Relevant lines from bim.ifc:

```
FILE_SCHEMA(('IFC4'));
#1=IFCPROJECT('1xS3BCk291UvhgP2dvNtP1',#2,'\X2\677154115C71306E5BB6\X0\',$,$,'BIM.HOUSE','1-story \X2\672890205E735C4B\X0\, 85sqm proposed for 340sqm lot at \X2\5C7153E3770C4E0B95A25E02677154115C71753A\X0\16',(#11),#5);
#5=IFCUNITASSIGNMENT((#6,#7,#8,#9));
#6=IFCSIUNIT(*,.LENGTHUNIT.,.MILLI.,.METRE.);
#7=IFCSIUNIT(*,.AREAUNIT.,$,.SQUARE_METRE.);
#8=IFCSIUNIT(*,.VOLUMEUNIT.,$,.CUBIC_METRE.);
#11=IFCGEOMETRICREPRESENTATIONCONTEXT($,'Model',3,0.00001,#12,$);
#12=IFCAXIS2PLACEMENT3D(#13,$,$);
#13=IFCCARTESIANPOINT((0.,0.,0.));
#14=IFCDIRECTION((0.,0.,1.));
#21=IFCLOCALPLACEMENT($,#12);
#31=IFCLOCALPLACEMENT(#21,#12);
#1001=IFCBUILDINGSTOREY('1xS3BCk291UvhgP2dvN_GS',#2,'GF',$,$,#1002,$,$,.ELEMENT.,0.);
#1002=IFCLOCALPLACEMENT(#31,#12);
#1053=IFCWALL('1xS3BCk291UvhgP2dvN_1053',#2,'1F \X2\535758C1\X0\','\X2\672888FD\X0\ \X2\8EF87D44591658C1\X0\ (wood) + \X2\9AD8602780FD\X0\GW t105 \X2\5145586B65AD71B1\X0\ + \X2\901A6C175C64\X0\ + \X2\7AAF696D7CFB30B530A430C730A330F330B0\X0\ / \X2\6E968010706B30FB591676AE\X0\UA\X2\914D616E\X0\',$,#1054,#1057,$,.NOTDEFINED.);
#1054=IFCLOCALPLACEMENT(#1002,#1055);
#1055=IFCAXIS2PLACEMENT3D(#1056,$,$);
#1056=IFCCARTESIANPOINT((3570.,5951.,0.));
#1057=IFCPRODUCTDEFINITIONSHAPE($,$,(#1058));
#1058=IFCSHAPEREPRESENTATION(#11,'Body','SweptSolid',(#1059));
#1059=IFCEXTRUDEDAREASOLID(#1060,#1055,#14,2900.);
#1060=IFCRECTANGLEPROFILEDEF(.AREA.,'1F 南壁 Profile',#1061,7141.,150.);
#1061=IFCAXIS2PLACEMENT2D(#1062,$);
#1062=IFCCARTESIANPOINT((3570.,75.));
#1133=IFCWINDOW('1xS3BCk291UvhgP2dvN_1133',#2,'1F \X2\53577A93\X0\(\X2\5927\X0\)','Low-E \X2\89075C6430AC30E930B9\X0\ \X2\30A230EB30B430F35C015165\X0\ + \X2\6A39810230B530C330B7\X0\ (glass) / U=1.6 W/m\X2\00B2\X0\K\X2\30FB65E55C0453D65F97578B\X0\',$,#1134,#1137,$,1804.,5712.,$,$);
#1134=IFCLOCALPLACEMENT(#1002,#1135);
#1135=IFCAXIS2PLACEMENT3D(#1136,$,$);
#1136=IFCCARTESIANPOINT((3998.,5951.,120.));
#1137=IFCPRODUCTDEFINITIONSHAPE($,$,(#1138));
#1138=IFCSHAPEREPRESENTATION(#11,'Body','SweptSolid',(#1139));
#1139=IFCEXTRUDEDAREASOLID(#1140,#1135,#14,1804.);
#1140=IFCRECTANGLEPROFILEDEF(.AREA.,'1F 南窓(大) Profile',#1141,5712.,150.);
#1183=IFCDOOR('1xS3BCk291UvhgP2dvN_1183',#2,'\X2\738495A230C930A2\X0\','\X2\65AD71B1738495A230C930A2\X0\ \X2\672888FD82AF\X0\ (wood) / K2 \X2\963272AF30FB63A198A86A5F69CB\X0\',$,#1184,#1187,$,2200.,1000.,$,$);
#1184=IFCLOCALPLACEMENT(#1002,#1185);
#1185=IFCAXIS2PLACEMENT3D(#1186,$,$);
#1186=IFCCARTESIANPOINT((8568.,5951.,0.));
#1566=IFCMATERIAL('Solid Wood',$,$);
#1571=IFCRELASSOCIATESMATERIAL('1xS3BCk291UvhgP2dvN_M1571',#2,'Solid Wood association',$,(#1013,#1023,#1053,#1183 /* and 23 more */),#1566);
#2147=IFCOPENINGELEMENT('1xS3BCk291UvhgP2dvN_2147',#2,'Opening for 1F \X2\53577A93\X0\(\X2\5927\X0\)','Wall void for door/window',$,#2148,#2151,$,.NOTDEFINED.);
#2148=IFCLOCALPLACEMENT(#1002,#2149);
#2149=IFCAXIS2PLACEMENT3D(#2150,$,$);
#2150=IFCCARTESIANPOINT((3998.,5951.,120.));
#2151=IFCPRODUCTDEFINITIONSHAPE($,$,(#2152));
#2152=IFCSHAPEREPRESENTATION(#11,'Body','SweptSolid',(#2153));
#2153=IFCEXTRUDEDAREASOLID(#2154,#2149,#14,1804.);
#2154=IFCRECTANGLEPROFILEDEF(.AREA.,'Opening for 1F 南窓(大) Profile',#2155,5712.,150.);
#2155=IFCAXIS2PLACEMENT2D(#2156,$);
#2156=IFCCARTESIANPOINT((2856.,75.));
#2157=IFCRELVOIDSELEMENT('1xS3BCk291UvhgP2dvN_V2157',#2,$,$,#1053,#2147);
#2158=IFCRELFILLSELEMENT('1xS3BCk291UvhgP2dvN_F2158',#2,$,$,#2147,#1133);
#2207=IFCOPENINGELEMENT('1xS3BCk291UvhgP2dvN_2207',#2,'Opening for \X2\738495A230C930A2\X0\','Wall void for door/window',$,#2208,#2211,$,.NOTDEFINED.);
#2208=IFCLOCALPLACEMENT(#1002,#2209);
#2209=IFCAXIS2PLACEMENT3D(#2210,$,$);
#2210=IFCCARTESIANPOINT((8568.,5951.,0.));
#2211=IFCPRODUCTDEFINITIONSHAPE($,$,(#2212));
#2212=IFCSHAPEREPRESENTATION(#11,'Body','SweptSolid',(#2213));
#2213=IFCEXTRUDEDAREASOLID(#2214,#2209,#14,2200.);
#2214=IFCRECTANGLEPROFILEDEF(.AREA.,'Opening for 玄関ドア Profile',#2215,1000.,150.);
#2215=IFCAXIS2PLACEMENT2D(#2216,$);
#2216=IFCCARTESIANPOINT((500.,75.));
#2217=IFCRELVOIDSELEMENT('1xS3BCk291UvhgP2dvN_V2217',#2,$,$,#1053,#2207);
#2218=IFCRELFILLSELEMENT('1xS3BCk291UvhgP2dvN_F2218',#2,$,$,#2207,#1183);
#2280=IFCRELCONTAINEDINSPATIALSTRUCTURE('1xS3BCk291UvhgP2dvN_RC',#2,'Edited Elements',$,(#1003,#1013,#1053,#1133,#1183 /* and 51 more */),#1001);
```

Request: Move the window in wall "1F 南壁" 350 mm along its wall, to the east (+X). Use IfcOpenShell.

```python
import ifcopenshell
import ifcopenshell.api.geometry
import ifcopenshell.util.placement

model = ifcopenshell.open("bim.ifc")

window = model.by_guid("1xS3BCk291UvhgP2dvN_1133")
opening = window.FillsVoids[0].RelatingOpeningElement
wall = opening.VoidsElements[0].RelatingBuildingElement

wall_matrix = ifcopenshell.util.placement.get_local_placement(wall.ObjectPlacement)
shift = wall_matrix[:3, 0] * 350.0
before = ifcopenshell.util.placement.get_local_placement(window.ObjectPlacement)[:3, 3].copy()

# The window is not placed relative to its opening, so move both.
for product in (opening, window):
    matrix = ifcopenshell.util.placement.get_local_placement(product.ObjectPlacement)
    matrix[:3, 3] += shift
    ifcopenshell.api.geometry.edit_object_placement(model, product=product, matrix=matrix, is_si=False)

after = ifcopenshell.util.placement.get_local_placement(window.ObjectPlacement)[:3, 3]
print("window moved by", (after - before).round(3) + 0.0)

model.write("bim_rev.ifc")
```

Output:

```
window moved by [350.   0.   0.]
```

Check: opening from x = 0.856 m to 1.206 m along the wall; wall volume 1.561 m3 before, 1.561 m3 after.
